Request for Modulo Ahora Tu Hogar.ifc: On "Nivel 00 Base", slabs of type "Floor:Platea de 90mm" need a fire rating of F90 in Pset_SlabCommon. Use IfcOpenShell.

First a look at what the model holds.

```python
import ifcopenshell
import ifcopenshell.util.element

model = ifcopenshell.open("Modulo Ahora Tu Hogar.ifc")
print(model.schema)
storey = next(s for s in model.by_type("IfcBuildingStorey") if s.Name == "Nivel 00 Base")
slabs = [e for e in ifcopenshell.util.element.get_decomposition(storey) if e.is_a("IfcSlab")]
seen = {}
for e in slabs:
    element_type = ifcopenshell.util.element.get_type(e)
    key = (element_type.Name if element_type != e and element_type else None, ifcopenshell.util.element.get_pset(e, "Pset_SlabCommon", "FireRating"))
    seen[key] = seen.get(key, 0) + 1
for (name, value), count in sorted(seen.items(), key=str):
    print(count, "x", name, "|", value)
```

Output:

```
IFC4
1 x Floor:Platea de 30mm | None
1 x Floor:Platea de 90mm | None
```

```python
import ifcopenshell
import ifcopenshell.api.pset
import ifcopenshell.util.element

model = ifcopenshell.open("Modulo Ahora Tu Hogar.ifc")

storey = next(s for s in model.by_type("IfcBuildingStorey") if s.Name == "Nivel 00 Base")
slabs = [e for e in ifcopenshell.util.element.get_decomposition(storey) if e.is_a("IfcSlab")]

count = 0
for e in slabs:
    element_type = ifcopenshell.util.element.get_type(e)
    if element_type in (None, e) or element_type.Name != "Floor:Platea de 90mm":
        continue
    # add_pset returns the element's existing set when there is one.
    pset = ifcopenshell.api.pset.add_pset(model, product=e, name="Pset_SlabCommon")
    ifcopenshell.api.pset.edit_pset(model, pset=pset, properties={"FireRating": "F90"})
    count += 1

print(count, "slabs updated")

model.write("Modulo Ahora Tu Hogar-out.ifc")
```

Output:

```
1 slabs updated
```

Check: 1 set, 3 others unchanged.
